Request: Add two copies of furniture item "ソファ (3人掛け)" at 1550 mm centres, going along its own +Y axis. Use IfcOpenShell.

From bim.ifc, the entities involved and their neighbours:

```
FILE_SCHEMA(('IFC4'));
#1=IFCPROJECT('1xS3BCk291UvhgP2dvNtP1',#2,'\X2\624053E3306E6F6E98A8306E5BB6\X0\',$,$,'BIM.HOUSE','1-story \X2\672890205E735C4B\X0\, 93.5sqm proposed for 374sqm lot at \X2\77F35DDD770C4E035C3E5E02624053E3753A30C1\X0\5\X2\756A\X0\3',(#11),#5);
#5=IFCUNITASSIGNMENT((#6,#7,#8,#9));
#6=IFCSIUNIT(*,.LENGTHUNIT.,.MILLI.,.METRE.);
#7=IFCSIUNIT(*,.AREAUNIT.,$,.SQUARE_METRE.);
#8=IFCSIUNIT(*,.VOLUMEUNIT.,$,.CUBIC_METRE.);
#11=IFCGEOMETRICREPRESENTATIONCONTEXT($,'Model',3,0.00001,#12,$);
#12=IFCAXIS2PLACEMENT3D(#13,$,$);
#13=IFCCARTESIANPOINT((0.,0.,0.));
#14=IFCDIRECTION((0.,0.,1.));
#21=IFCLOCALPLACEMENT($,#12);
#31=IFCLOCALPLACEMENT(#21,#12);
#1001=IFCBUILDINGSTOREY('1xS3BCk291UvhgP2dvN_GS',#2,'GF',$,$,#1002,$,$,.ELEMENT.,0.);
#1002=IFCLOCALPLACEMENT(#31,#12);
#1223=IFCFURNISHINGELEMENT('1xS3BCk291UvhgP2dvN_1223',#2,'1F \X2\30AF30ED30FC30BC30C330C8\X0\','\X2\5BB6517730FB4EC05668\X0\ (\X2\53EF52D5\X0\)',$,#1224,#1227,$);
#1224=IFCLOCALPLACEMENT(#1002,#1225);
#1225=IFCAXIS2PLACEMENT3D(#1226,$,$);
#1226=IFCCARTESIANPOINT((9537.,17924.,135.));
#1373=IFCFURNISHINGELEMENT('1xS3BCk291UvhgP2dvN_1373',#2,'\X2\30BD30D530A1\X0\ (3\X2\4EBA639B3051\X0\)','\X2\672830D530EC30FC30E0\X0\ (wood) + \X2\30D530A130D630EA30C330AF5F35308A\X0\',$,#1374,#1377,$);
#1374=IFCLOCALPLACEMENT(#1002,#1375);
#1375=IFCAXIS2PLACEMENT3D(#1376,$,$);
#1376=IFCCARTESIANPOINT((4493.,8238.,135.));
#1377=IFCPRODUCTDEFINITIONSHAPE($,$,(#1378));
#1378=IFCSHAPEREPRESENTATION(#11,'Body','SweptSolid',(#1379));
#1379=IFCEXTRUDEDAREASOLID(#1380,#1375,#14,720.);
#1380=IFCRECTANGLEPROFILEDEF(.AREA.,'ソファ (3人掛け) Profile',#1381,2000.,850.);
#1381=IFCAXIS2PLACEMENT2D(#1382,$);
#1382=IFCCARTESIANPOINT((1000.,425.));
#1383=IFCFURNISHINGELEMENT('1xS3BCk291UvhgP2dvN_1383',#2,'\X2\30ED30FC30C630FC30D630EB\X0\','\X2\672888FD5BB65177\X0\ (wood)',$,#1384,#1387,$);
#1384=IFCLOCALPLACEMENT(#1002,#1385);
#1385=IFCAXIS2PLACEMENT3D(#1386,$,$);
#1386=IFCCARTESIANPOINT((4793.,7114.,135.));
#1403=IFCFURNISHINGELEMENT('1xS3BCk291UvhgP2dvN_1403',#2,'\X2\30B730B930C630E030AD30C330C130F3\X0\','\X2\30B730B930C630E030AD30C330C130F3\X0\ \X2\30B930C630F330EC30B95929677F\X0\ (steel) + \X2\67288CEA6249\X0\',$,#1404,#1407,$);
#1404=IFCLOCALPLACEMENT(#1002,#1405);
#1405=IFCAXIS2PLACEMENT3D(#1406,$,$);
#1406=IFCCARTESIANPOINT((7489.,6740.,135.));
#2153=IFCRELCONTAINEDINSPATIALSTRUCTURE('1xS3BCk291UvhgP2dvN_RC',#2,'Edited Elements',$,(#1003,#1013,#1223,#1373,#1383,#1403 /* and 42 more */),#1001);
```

```python
import ifcopenshell
import ifcopenshell.api.geometry
import ifcopenshell.api.root
import ifcopenshell.util.element
import ifcopenshell.util.placement
import ifcopenshell.util.unit

model = ifcopenshell.open("bim.ifc")
unit_scale = ifcopenshell.util.unit.calculate_unit_scale(model)


def reuse_history(source, copy):
    """copy_class also copies each property set's owner history, people and application; keep the originals."""
    for rel in copy.IsDefinedBy:
        if rel.is_a("IfcRelDefinesByProperties") and (history := rel.RelatingPropertyDefinition.OwnerHistory):
            rel.RelatingPropertyDefinition.OwnerHistory = source.OwnerHistory
            ifcopenshell.util.element.remove_deep2(model, history)


source = model.by_guid("1xS3BCk291UvhgP2dvN_1373")
base = ifcopenshell.util.placement.get_local_placement(source.ObjectPlacement)
step = base[:3, 1] * 1.55 / unit_scale

for i in range(1, 3):
    copy = ifcopenshell.api.root.copy_class(model, product=source)
    copy.Representation = ifcopenshell.util.element.copy_deep(
        model, source.Representation, exclude=["IfcGeometricRepresentationContext", "IfcRepresentationMap"]
    )
    reuse_history(source, copy)
    matrix = base.copy()
    matrix[:3, 3] += i * step
    print("added at", matrix[:3, 3].round(3) + 0.0)
    ifcopenshell.api.geometry.edit_object_placement(model, product=copy, matrix=matrix, is_si=False)

model.write("bim_v2.ifc")
```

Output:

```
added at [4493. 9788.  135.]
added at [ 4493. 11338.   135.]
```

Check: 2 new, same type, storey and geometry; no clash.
